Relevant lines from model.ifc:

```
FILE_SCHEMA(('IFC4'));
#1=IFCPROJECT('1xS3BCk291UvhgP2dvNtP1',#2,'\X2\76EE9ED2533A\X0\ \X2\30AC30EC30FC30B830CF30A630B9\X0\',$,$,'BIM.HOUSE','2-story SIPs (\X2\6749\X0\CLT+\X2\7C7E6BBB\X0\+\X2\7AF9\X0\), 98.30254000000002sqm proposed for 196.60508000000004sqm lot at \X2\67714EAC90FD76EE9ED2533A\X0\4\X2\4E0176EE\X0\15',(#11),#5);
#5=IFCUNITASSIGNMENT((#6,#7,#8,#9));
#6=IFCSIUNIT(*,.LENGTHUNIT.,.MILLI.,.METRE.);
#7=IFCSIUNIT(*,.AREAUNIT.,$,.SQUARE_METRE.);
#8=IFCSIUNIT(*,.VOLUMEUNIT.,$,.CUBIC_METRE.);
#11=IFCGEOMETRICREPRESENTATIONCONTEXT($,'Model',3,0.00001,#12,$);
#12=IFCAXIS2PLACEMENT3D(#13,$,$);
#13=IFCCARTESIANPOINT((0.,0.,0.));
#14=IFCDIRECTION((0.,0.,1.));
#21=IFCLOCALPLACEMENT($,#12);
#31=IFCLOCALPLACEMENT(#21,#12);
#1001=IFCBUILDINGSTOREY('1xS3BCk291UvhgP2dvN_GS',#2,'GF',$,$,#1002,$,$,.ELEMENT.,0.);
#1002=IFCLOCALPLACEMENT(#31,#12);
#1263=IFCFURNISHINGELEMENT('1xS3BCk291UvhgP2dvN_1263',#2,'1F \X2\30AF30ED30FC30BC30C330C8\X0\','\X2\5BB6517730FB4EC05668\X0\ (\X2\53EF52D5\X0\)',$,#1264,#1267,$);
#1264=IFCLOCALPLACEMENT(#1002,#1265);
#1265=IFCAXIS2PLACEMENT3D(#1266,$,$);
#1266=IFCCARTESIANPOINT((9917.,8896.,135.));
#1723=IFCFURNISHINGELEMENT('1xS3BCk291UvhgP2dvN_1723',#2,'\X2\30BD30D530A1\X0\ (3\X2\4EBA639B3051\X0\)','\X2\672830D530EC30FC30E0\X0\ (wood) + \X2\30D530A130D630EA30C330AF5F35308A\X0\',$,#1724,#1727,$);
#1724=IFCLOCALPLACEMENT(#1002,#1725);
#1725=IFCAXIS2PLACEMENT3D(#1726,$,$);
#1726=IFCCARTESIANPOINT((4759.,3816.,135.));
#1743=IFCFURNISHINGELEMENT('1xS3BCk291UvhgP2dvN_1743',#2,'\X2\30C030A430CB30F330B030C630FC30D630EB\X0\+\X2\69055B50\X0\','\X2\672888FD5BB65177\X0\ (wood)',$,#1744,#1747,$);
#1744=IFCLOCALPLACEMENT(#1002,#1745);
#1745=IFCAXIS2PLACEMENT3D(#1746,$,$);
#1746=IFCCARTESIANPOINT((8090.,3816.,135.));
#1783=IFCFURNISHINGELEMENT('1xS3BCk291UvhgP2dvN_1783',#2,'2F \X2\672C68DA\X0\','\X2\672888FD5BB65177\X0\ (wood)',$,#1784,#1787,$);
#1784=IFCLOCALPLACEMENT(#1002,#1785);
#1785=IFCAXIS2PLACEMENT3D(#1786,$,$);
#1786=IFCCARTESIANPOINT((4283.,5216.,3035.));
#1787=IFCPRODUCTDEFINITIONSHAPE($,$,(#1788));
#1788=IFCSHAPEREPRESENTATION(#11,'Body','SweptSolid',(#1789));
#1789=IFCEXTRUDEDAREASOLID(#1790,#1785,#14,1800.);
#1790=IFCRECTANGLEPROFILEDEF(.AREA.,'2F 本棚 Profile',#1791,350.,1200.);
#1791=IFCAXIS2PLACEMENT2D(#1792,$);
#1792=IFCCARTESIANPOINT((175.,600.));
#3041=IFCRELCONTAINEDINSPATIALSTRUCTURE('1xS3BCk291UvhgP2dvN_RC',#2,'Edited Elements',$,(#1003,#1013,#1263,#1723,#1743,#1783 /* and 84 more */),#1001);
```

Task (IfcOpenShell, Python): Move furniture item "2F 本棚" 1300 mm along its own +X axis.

```python
import ifcopenshell
import ifcopenshell.api.geometry
import ifcopenshell.util.placement
import ifcopenshell.util.unit

model = ifcopenshell.open("model.ifc")
unit_scale = ifcopenshell.util.unit.calculate_unit_scale(model)

item = model.by_id(1783)
matrix = ifcopenshell.util.placement.get_local_placement(item.ObjectPlacement)
matrix[:3, 3] += matrix[:3, 0] * 1.3 / unit_scale
ifcopenshell.api.geometry.edit_object_placement(model, product=item, matrix=matrix, is_si=False)

print(ifcopenshell.util.placement.get_local_placement(item.ObjectPlacement).round(3) + 0.0)

model.write("model_rev.ifc")
```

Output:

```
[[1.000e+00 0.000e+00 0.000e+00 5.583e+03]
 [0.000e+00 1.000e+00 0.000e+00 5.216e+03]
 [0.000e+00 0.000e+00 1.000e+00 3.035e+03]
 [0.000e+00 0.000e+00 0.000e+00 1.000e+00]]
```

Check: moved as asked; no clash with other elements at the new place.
